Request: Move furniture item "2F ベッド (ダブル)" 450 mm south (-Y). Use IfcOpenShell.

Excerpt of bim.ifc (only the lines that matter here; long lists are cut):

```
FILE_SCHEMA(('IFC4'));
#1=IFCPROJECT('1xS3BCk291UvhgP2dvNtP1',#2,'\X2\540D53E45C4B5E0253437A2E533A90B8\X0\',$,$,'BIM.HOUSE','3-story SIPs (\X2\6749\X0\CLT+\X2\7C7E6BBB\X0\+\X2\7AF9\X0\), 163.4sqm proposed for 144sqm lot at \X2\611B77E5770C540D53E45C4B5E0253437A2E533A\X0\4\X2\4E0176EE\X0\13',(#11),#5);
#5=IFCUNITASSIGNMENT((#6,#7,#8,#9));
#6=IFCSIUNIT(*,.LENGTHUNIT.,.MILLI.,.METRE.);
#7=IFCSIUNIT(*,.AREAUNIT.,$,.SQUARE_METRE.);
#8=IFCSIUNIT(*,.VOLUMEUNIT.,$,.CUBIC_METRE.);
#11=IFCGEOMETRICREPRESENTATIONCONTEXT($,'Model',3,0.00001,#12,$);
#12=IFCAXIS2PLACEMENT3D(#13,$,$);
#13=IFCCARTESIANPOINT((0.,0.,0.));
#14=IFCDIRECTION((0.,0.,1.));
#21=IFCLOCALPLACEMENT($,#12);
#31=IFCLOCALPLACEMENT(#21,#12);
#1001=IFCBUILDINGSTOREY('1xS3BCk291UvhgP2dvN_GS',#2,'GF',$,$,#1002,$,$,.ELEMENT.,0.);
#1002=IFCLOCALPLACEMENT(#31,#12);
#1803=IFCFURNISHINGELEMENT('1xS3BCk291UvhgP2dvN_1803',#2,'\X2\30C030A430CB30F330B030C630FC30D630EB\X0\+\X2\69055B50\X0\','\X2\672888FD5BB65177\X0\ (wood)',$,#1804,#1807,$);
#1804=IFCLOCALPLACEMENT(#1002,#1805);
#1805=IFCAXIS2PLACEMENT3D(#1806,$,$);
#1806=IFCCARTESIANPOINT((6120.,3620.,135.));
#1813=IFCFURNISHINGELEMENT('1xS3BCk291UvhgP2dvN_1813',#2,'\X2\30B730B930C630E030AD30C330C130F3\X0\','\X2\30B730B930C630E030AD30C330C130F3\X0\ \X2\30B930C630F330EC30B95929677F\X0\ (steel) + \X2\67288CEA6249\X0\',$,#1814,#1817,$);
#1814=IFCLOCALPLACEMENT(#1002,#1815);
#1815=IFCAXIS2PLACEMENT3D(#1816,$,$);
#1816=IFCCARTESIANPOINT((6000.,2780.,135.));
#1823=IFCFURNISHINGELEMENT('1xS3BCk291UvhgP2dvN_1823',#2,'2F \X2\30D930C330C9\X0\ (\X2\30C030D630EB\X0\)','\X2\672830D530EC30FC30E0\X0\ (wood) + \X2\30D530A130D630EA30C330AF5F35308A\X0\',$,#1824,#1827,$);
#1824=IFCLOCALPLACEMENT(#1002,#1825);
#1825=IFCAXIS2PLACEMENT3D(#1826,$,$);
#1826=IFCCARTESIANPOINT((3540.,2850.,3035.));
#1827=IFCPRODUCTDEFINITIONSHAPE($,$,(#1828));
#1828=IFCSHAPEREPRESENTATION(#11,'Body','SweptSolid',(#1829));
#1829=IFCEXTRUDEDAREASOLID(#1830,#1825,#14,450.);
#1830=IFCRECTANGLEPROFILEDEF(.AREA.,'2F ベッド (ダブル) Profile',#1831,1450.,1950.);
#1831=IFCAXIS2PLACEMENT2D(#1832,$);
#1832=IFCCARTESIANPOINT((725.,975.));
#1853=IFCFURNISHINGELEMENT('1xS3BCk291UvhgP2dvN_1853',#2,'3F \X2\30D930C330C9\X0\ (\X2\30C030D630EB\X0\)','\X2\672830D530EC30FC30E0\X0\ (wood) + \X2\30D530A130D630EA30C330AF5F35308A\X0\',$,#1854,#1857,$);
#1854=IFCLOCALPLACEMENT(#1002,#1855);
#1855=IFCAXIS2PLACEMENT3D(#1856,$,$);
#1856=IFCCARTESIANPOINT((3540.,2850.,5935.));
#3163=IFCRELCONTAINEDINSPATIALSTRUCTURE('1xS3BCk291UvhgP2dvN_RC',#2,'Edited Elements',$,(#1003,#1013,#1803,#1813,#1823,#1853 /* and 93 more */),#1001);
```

```python
import ifcopenshell
import ifcopenshell.api.geometry
import ifcopenshell.util.placement
import ifcopenshell.util.unit

model = ifcopenshell.open("bim.ifc")
unit_scale = ifcopenshell.util.unit.calculate_unit_scale(model)

item = model.by_guid("1xS3BCk291UvhgP2dvN_1823")
matrix = ifcopenshell.util.placement.get_local_placement(item.ObjectPlacement)
matrix[1, 3] -= 0.45 / unit_scale
ifcopenshell.api.geometry.edit_object_placement(model, product=item, matrix=matrix, is_si=False)

print(ifcopenshell.util.placement.get_local_placement(item.ObjectPlacement).round(3) + 0.0)

model.write("bim_updated.ifc")
```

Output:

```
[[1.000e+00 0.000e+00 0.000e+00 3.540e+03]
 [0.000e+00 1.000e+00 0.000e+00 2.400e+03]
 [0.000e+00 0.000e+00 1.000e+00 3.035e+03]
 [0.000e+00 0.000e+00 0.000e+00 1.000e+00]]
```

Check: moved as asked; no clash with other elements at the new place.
